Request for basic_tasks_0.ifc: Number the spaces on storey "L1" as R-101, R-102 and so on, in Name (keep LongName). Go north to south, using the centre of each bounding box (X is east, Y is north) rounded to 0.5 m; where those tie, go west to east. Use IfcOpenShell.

First a look at what the model holds.

```python
import ifcopenshell
import ifcopenshell.util.element
import ifcopenshell.util.placement

model = ifcopenshell.open("basic_tasks_0.ifc")
print(model.schema)
storey = next(s for s in model.by_type("IfcBuildingStorey") if s.Name == "L1")
spaces = [e for e in ifcopenshell.util.element.get_decomposition(storey) if e.is_a("IfcSpace")]
for e in sorted(spaces, key=lambda e: e.id()):
    origin = ifcopenshell.util.placement.get_local_placement(e.ObjectPlacement)[:3, 3]
    print(e.id(), e.Name, e.LongName, origin.round(2) + 0.0, sep=" | ")
```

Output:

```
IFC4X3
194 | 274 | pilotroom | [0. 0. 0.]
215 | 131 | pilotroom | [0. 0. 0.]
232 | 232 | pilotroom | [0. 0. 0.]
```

```python
import ifcopenshell
import ifcopenshell.geom
import ifcopenshell.util.element
import ifcopenshell.util.shape

model = ifcopenshell.open("basic_tasks_0.ifc")
settings = ifcopenshell.geom.settings()
settings.set("use-world-coords", True)


def centre(element):
    shape = ifcopenshell.geom.create_shape(settings, element)
    return ifcopenshell.util.shape.get_bbox_centroid(shape.geometry)


storey = next(s for s in model.by_type("IfcBuildingStorey") if s.Name == "L1")
spaces = [e for e in ifcopenshell.util.element.get_decomposition(storey) if e.is_a("IfcSpace")]

# Insertion points can sit at a corner or the storey origin, so sort by the geometry (in metres).
centres = {e: centre(e) for e in spaces}
spaces.sort(key=lambda e: (-round(centres[e][1] / 0.5), centres[e][0]))

for i, e in enumerate(spaces, start=1):
    number = f"R-1{i:02d}"
    e.Name = number
    print(e.id(), number)

model.write("basic_tasks_0_rev.ifc")
```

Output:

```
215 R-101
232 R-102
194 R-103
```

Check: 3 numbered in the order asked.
